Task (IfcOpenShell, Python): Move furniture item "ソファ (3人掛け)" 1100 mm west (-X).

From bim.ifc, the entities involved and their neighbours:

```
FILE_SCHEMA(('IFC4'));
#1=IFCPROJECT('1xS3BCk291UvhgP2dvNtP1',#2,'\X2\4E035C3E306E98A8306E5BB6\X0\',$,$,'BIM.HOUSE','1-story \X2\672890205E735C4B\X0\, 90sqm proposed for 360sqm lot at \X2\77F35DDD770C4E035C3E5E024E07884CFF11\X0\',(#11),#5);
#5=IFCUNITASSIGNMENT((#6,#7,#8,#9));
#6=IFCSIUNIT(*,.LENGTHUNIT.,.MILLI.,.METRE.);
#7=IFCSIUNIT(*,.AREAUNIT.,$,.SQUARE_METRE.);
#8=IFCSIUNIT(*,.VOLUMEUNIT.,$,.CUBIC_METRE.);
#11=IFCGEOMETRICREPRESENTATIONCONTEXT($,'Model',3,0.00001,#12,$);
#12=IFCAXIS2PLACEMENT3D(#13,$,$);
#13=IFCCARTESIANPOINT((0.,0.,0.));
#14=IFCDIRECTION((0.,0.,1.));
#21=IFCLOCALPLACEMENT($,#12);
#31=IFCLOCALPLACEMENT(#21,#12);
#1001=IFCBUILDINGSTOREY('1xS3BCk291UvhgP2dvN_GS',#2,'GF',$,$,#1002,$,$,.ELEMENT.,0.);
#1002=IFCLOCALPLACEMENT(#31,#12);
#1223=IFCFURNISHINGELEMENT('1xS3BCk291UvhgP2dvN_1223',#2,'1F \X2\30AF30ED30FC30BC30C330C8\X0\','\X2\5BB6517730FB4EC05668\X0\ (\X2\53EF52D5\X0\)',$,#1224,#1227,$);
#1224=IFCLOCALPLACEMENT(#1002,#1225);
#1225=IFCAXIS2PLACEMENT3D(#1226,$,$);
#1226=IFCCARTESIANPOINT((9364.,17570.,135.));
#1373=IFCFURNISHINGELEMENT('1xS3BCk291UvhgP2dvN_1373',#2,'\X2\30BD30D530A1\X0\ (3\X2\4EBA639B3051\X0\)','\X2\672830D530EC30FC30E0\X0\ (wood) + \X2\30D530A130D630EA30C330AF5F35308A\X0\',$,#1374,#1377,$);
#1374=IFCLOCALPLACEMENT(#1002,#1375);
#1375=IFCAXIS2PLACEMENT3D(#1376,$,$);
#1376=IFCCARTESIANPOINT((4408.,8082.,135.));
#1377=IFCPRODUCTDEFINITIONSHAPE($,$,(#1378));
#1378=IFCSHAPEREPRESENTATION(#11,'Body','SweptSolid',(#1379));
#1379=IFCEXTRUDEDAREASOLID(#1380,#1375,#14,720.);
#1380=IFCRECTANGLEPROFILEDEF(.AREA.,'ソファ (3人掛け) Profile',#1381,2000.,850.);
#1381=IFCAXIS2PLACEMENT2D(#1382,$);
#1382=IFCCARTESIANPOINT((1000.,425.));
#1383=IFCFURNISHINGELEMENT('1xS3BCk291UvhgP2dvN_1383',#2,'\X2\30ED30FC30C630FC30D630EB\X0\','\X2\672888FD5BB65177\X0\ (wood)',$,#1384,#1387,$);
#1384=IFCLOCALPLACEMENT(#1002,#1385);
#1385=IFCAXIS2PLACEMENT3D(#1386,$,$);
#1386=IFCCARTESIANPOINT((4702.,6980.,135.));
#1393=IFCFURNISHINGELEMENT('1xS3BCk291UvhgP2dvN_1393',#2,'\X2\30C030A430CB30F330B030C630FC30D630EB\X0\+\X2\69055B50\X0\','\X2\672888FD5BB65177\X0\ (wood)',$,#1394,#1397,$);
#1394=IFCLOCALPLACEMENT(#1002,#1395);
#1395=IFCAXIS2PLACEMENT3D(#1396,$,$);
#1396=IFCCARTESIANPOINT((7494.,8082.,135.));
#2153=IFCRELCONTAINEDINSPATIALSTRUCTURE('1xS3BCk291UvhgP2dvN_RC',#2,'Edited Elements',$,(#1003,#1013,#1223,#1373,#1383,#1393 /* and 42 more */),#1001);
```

```python
import ifcopenshell
import ifcopenshell.api.geometry
import ifcopenshell.util.placement

model = ifcopenshell.open("bim.ifc")

item = model.by_guid("1xS3BCk291UvhgP2dvN_1373")
matrix = ifcopenshell.util.placement.get_local_placement(item.ObjectPlacement)
matrix[0, 3] -= 1100.0
ifcopenshell.api.geometry.edit_object_placement(model, product=item, matrix=matrix, is_si=False)

print(ifcopenshell.util.placement.get_local_placement(item.ObjectPlacement).round(3) + 0.0)

model.write("bim_rev.ifc")
```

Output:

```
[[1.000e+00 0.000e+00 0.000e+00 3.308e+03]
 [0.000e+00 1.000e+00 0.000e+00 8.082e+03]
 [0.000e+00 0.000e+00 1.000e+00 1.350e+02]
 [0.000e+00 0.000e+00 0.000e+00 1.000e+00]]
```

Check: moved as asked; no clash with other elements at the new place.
